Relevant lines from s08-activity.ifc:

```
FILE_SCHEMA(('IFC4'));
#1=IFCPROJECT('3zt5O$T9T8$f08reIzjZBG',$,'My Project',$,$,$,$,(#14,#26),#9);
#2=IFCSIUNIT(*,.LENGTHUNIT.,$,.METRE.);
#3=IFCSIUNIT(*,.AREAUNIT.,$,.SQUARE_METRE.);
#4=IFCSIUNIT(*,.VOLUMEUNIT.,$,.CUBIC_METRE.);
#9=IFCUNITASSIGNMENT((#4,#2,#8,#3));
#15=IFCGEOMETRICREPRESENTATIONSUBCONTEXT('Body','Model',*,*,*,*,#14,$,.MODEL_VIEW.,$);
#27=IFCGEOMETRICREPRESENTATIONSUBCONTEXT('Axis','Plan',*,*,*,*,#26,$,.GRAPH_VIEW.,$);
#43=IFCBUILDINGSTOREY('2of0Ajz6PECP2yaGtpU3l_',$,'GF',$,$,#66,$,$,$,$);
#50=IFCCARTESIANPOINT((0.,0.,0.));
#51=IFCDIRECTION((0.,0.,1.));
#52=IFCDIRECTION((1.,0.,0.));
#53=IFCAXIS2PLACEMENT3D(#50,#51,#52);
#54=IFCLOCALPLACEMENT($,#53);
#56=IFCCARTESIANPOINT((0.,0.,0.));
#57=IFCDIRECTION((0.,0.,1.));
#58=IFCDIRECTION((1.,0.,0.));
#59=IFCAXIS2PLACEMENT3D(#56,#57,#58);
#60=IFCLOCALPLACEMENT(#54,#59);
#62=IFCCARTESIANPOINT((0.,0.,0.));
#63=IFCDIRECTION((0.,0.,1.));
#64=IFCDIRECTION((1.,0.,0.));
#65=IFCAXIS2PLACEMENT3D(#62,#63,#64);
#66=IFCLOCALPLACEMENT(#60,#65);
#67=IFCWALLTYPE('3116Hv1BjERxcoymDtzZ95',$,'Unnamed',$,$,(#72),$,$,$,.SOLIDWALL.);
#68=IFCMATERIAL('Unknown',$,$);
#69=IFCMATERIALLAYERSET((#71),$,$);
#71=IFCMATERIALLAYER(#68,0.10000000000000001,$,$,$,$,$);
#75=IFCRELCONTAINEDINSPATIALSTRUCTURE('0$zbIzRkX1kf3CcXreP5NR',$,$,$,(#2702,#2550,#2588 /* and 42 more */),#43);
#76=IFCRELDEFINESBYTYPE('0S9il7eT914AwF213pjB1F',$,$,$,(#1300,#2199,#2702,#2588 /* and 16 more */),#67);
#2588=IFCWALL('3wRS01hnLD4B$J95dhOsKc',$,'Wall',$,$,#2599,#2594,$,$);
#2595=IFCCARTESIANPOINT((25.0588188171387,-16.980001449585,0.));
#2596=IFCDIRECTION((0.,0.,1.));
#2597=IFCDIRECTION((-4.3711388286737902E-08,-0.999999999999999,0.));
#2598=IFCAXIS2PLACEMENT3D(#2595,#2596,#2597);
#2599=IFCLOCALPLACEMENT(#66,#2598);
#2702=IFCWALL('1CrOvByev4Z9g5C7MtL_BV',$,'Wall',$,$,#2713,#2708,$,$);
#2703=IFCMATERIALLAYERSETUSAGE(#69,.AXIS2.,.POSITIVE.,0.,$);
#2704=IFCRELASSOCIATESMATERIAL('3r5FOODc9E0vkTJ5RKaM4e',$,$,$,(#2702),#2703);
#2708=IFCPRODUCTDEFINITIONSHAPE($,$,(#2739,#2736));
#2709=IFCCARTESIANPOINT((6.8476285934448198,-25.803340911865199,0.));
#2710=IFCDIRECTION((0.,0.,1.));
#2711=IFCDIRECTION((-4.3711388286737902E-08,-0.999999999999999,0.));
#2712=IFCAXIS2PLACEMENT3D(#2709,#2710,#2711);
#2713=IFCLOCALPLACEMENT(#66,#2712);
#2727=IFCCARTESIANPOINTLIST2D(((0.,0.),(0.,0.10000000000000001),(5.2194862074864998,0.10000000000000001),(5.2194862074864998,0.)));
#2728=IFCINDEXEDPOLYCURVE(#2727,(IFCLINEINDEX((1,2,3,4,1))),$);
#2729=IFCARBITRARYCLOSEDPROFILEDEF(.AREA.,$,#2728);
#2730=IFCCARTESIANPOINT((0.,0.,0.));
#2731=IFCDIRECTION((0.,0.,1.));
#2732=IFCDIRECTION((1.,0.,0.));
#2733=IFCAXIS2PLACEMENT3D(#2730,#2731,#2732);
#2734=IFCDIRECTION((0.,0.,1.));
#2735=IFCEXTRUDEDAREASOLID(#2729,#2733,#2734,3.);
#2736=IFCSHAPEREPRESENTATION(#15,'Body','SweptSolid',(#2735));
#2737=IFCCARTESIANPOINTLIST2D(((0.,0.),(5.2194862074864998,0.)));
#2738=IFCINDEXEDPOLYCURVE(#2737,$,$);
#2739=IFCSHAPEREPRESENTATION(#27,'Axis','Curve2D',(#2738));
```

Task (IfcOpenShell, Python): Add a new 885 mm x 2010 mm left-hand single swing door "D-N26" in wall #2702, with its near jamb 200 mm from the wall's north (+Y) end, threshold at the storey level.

```python
import numpy as np
import ifcopenshell
import ifcopenshell.api.feature
import ifcopenshell.api.geometry
import ifcopenshell.api.root
import ifcopenshell.api.spatial
import ifcopenshell.geom
import ifcopenshell.util.element
import ifcopenshell.util.placement
import ifcopenshell.util.representation
import ifcopenshell.util.shape
import ifcopenshell.util.unit

model = ifcopenshell.open("s08-activity.ifc")
unit_scale = ifcopenshell.util.unit.calculate_unit_scale(model)
settings = ifcopenshell.geom.settings()


def volume(element):
    """Net volume in cubic metres, openings subtracted."""
    shape = ifcopenshell.geom.create_shape(settings, element)
    return ifcopenshell.util.shape.get_volume(shape.geometry)


wall = model.by_guid("1CrOvByev4Z9g5C7MtL_BV")
storey = ifcopenshell.util.element.get_container(wall, ifc_class="IfcBuildingStorey")
context = ifcopenshell.util.representation.get_context(model, "Model", "Body", "MODEL_VIEW")
before = volume(wall)

width, height, from_end, sill = 0.885, 2.01, 0.2, 0.0  # metres

# The wall runs along its own X axis, and the end named is its -X end.
wall_shape = ifcopenshell.geom.create_shape(settings, wall)
x, y, z = ifcopenshell.util.shape.get_vertices(wall_shape.geometry).T
start = x.min() + from_end
face, thickness = float(y.min()), float(y.max() - y.min())
wall_matrix = ifcopenshell.util.placement.get_local_placement(wall.ObjectPlacement)
level = ifcopenshell.util.placement.get_local_placement(storey.ObjectPlacement)[2, 3]


def in_wall(x, y):
    """Placement at x, y metres in the wall's axes, at sill height."""
    matrix = wall_matrix.copy()
    matrix[:, 3] = wall_matrix @ np.array([x / unit_scale, y / unit_scale, 0.0, 1.0])
    matrix[2, 3] = level + sill / unit_scale
    return matrix


# Opening: a box that overshoots both wall faces by 50 mm.
opening = ifcopenshell.api.root.create_entity(model, ifc_class="IfcOpeningElement", predefined_type="OPENING")
box = ifcopenshell.api.geometry.add_wall_representation(
    model, context=context, length=width, height=height, thickness=thickness + 0.1
)
ifcopenshell.api.geometry.assign_representation(model, product=opening, representation=box)
ifcopenshell.api.geometry.edit_object_placement(model, product=opening, matrix=in_wall(start, face - 0.05), is_si=False)
ifcopenshell.api.feature.add_feature(model, feature=opening, element=wall)

door = ifcopenshell.api.root.create_entity(model, ifc_class="IfcDoor", name="D-N26", predefined_type="DOOR")
door.OverallWidth, door.OverallHeight = width / unit_scale, height / unit_scale
door.OperationType = "SINGLE_SWING_LEFT"
body = ifcopenshell.api.geometry.add_door_representation(
    model,
    context=context,
    overall_width=door.OverallWidth,
    overall_height=door.OverallHeight,
    operation_type="SINGLE_SWING_LEFT",
    lining_properties={"LiningDepth": thickness / unit_scale, "ThresholdDepth": thickness / unit_scale},
)
ifcopenshell.api.geometry.assign_representation(model, product=door, representation=body)
ifcopenshell.api.spatial.assign_container(model, products=[door], relating_structure=storey)
ifcopenshell.api.feature.add_filling(model, opening=opening, element=door)

# The lining spans the wall, so the door starts at the wall face.
ifcopenshell.api.geometry.edit_object_placement(model, product=door, matrix=in_wall(start, face), is_si=False)

after = volume(wall)

print(f"wall volume {before:.3f} -> {after:.3f} m3")

model.write("s08-activity_rev.ifc")
```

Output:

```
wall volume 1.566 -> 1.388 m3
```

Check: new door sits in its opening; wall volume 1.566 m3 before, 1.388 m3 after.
